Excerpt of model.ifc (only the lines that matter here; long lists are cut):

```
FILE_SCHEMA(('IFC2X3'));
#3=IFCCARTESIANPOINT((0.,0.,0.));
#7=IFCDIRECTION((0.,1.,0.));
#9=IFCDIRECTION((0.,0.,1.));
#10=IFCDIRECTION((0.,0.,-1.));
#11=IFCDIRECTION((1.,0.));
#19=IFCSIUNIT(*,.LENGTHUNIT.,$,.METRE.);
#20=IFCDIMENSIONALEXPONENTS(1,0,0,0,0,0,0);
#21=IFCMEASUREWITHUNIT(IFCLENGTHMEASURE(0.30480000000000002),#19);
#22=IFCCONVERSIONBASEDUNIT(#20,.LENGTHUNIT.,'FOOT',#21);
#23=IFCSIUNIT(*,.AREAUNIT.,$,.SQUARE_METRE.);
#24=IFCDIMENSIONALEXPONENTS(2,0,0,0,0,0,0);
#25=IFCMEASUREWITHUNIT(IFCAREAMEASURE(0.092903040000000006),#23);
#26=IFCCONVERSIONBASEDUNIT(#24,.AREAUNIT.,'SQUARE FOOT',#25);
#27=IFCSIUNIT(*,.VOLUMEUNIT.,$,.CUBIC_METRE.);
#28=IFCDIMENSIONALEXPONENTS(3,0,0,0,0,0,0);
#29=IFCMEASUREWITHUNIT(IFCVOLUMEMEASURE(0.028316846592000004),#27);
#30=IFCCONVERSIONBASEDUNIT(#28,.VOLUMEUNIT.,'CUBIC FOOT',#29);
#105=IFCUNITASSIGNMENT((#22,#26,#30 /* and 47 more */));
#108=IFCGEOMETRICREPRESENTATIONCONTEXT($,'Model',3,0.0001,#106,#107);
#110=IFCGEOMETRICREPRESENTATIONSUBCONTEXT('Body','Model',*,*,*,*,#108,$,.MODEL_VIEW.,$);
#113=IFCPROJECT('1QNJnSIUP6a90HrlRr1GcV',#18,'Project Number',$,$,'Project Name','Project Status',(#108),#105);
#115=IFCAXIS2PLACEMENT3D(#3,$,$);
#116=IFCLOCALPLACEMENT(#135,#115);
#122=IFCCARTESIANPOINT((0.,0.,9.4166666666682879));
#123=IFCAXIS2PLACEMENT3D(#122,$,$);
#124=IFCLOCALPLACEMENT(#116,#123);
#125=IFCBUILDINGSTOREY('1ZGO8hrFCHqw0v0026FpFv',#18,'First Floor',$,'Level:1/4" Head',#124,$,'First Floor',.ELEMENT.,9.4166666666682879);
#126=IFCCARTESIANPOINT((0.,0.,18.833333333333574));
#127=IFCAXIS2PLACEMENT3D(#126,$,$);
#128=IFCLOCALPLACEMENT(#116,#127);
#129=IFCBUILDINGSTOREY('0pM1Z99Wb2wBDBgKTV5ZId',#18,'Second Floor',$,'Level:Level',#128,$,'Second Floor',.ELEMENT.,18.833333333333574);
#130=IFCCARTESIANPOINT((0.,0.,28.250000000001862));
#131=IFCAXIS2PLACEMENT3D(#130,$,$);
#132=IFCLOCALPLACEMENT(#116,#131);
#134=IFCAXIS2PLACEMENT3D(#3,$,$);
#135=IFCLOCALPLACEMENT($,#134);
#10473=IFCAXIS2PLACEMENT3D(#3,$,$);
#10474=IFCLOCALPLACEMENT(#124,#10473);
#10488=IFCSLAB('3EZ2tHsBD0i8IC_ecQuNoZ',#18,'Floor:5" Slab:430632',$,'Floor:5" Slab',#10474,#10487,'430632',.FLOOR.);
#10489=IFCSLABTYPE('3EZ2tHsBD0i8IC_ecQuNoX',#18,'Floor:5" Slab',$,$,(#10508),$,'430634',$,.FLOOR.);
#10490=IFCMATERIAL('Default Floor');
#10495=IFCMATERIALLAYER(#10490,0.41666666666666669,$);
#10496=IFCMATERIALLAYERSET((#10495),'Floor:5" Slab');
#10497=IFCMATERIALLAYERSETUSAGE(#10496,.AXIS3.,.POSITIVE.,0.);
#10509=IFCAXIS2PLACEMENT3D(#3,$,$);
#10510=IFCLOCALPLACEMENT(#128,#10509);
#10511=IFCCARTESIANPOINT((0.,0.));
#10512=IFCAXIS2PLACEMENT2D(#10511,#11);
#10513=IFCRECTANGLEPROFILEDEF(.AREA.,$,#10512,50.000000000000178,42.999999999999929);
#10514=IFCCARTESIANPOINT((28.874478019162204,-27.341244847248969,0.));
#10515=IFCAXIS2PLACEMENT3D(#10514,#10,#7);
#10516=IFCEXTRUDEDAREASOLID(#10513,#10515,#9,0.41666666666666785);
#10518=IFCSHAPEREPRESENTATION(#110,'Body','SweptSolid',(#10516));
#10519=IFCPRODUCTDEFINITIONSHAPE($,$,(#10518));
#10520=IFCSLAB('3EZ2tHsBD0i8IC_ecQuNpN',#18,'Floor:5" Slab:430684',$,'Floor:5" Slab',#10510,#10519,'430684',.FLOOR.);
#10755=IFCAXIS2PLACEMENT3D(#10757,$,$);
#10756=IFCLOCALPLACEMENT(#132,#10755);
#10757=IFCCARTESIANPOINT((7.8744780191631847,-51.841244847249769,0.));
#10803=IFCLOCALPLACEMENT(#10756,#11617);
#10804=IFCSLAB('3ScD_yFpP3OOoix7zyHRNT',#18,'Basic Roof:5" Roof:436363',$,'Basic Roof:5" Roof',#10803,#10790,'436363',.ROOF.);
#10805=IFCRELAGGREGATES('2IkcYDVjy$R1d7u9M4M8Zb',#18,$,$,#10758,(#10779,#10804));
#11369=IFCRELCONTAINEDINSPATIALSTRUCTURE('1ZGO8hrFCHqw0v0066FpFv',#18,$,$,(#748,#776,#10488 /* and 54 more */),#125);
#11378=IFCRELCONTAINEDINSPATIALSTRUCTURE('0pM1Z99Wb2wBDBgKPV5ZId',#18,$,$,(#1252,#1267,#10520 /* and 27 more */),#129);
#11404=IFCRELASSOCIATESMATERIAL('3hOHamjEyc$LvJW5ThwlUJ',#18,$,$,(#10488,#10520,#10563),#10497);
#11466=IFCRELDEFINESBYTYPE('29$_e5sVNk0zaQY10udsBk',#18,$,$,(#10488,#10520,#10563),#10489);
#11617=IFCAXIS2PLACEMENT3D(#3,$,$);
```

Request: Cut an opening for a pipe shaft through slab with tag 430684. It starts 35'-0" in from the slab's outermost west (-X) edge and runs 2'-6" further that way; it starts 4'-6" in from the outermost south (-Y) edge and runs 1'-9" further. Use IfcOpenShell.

```python
import numpy as np
import ifcopenshell
import ifcopenshell.api.feature
import ifcopenshell.api.geometry
import ifcopenshell.api.root
import ifcopenshell.geom
import ifcopenshell.util.placement
import ifcopenshell.util.representation
import ifcopenshell.util.shape
import ifcopenshell.util.unit

model = ifcopenshell.open("model.ifc")
unit_scale = ifcopenshell.util.unit.calculate_unit_scale(model)
settings = ifcopenshell.geom.settings()


def volume(element):
    """Net volume in cubic metres, openings subtracted."""
    shape = ifcopenshell.geom.create_shape(settings, element)
    return ifcopenshell.util.shape.get_volume(shape.geometry)


slab = model.by_guid("3EZ2tHsBD0i8IC_ecQuNpN")
before = volume(slab)

# Extent in the slab's own axes, in metres. The edges named are its -X and -Y sides.
slab_shape = ifcopenshell.geom.create_shape(settings, slab)
vertices = ifcopenshell.util.shape.get_vertices(slab_shape.geometry)
x_min, y_min, bottom = vertices.min(axis=0)
top = vertices[:, 2].max()

opening = ifcopenshell.api.root.create_entity(model, ifc_class="IfcOpeningElement", name="Pipe shaft opening")
context = ifcopenshell.util.representation.get_context(model, "Model", "Body", "MODEL_VIEW")
width, depth = 0.762, 0.5334
outline = [(0.0, 0.0), (width, 0.0), (width, depth), (0.0, depth), (0.0, 0.0)]
# Overshoot both faces by 50 mm so the cut is clean.
shape = ifcopenshell.api.geometry.add_slab_representation(
    model, context=context, depth=top - bottom + 0.1, polyline=outline
)
ifcopenshell.api.geometry.assign_representation(model, product=opening, representation=shape)

matrix = ifcopenshell.util.placement.get_local_placement(slab.ObjectPlacement)
matrix[:, 3] = matrix @ np.append(np.array([x_min + 10.668, y_min + 1.3716, bottom - 0.05]) / unit_scale, 1.0)
ifcopenshell.api.geometry.edit_object_placement(model, product=opening, matrix=matrix, is_si=False)
ifcopenshell.api.feature.add_feature(model, feature=opening, element=slab)

after = volume(slab)

print(f"slab volume {before:.3f} -> {after:.3f} m3")

model.write("model_updated.ifc")
```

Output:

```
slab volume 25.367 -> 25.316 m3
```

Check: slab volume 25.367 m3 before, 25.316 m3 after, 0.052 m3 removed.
